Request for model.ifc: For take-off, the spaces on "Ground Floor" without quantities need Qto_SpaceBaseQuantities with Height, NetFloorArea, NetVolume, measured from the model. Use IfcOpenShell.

First a look at what the model holds.

```python
import ifcopenshell
import ifcopenshell.util.element
import ifcopenshell.util.unit

model = ifcopenshell.open("model.ifc")
print(model.schema)
for unit_type in ("LENGTHUNIT", "AREAUNIT", "VOLUMEUNIT"):
    print(unit_type, ifcopenshell.util.unit.calculate_unit_scale(model, unit_type))
storey = next(s for s in model.by_type("IfcBuildingStorey") if s.Name == "Ground Floor")
spaces = [e for e in ifcopenshell.util.element.get_decomposition(storey) if e.is_a("IfcSpace")]
for e in sorted(spaces, key=lambda e: e.id()):
    print(e.id(), e.is_a(), e.Name, list(ifcopenshell.util.element.get_psets(e, qtos_only=True)), sep=" | ")
```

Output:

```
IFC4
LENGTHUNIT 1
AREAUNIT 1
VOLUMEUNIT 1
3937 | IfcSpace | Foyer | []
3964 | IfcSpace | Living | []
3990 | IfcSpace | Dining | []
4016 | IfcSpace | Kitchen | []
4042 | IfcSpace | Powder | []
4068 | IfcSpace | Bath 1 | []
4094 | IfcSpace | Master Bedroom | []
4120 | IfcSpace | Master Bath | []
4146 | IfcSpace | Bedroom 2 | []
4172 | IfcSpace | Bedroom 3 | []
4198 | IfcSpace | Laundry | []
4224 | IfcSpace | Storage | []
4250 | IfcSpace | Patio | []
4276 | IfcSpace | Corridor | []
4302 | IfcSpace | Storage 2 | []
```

```python
import ifcopenshell
import ifcopenshell.api.pset
import ifcopenshell.geom
import ifcopenshell.util.element
import ifcopenshell.util.shape
import ifcopenshell.util.unit

model = ifcopenshell.open("model.ifc")
unit_scale = ifcopenshell.util.unit.calculate_unit_scale(model)
area_scale = ifcopenshell.util.unit.calculate_unit_scale(model, "AREAUNIT")
volume_scale = ifcopenshell.util.unit.calculate_unit_scale(model, "VOLUMEUNIT")
settings = ifcopenshell.geom.settings()

storey = next(s for s in model.by_type("IfcBuildingStorey") if s.Name == "Ground Floor")
spaces = [e for e in ifcopenshell.util.element.get_decomposition(storey) if e.is_a("IfcSpace")]

for e in sorted(spaces, key=lambda e: e.id()):
    if ifcopenshell.util.element.get_psets(e, qtos_only=True, should_inherit=False):
        continue
    # Geometry comes back in metres, in the element's own axes.
    shape = ifcopenshell.geom.create_shape(settings, e)
    values = {
        "Height": ifcopenshell.util.shape.get_z(shape.geometry) / unit_scale,
        "NetFloorArea": ifcopenshell.util.shape.get_footprint_area(shape.geometry) / area_scale,
        "NetVolume": ifcopenshell.util.shape.get_volume(shape.geometry) / volume_scale,
    }
    qto = ifcopenshell.api.pset.add_qto(model, product=e, name="Qto_SpaceBaseQuantities")
    ifcopenshell.api.pset.edit_qto(model, qto=qto, properties=values)
    print(e.id(), {k: round(v, 3) for k, v in values.items()})

model.write("model_updated.ifc")
```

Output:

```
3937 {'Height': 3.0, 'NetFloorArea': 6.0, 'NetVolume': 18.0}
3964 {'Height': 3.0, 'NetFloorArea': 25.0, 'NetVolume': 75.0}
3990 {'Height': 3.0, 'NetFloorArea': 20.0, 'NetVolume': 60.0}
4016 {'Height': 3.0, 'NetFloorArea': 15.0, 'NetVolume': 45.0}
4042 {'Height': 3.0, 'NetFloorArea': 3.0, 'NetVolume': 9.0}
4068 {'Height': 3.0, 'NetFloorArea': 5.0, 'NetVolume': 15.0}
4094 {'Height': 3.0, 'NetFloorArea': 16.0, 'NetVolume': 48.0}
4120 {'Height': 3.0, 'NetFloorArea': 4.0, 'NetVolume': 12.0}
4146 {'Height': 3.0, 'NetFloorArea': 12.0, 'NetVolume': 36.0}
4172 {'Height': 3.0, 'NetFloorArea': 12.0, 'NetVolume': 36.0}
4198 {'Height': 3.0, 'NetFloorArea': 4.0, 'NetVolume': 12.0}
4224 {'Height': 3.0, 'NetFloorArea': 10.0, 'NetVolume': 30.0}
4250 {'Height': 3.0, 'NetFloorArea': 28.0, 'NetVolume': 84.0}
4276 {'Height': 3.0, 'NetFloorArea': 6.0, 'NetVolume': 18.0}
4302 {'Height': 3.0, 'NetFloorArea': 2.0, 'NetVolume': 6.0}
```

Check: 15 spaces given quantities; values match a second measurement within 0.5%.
